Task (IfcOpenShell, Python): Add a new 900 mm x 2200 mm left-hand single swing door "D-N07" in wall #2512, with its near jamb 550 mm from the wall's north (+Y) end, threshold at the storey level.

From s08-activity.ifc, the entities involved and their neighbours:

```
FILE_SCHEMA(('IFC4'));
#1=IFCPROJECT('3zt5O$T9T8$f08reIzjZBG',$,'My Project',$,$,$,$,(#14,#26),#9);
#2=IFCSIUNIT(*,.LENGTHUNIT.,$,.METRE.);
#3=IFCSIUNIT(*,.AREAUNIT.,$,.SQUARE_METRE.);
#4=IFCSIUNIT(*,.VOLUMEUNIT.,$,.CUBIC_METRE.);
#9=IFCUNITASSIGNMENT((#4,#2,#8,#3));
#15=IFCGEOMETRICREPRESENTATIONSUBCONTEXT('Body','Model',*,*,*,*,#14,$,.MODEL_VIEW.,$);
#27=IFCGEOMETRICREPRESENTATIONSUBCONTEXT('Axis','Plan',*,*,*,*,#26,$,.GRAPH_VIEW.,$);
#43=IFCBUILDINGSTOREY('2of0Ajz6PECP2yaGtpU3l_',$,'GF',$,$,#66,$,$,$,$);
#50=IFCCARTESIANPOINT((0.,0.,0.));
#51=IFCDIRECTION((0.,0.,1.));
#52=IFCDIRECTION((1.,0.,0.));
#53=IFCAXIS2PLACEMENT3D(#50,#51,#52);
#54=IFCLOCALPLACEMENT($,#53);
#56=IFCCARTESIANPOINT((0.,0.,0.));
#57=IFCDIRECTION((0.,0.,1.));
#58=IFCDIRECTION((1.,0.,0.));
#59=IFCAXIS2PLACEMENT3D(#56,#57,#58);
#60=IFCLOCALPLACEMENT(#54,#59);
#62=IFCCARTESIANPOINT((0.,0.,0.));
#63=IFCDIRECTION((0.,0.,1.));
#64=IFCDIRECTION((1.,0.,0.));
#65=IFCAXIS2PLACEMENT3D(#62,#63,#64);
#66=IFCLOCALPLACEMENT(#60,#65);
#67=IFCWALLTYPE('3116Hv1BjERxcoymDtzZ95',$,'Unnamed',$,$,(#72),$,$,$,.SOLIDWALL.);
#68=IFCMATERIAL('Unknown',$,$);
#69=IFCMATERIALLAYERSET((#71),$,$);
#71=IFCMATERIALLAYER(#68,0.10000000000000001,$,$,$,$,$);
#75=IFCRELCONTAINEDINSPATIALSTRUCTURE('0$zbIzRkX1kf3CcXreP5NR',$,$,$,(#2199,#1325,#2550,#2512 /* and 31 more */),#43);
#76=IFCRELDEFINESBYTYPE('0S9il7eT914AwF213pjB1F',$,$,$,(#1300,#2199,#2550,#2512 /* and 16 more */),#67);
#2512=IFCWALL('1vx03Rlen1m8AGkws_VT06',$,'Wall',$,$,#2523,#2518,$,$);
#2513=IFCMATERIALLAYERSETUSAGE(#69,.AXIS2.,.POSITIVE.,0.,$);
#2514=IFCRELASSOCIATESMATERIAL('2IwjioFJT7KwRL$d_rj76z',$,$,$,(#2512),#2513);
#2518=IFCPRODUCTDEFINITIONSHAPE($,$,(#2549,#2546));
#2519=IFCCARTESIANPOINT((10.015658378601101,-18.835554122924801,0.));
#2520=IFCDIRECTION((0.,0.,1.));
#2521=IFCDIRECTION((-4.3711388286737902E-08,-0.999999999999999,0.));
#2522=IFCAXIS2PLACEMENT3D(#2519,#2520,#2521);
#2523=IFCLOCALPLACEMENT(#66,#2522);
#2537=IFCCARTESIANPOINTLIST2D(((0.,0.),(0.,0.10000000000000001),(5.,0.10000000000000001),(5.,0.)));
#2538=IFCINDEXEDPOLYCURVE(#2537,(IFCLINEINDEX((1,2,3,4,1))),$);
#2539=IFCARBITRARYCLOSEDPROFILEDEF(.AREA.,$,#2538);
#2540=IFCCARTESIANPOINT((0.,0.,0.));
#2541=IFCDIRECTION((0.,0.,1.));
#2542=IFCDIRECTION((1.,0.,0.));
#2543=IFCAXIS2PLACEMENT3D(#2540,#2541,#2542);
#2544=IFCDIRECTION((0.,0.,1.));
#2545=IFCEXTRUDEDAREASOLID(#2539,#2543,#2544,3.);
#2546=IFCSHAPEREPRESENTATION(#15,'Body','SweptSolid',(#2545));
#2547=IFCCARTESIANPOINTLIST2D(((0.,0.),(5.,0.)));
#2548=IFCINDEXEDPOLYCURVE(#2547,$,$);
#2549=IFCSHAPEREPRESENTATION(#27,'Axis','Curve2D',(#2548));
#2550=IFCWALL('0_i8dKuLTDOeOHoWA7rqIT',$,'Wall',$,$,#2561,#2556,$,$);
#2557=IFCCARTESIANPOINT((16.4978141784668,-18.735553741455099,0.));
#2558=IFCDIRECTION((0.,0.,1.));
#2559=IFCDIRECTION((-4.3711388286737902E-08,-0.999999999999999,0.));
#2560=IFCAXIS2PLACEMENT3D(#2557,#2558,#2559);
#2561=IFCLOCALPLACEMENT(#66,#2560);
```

```python
import numpy as np
import ifcopenshell
import ifcopenshell.api.feature
import ifcopenshell.api.geometry
import ifcopenshell.api.root
import ifcopenshell.api.spatial
import ifcopenshell.geom
import ifcopenshell.util.element
import ifcopenshell.util.placement
import ifcopenshell.util.representation
import ifcopenshell.util.shape
import ifcopenshell.util.unit

model = ifcopenshell.open("s08-activity.ifc")
unit_scale = ifcopenshell.util.unit.calculate_unit_scale(model)
settings = ifcopenshell.geom.settings()


def volume(element):
    """Net volume in cubic metres, openings subtracted."""
    shape = ifcopenshell.geom.create_shape(settings, element)
    return ifcopenshell.util.shape.get_volume(shape.geometry)


wall = model.by_id(2512)
storey = ifcopenshell.util.element.get_container(wall, ifc_class="IfcBuildingStorey")
context = ifcopenshell.util.representation.get_context(model, "Model", "Body", "MODEL_VIEW")
before = volume(wall)

width, height, from_end, sill = 0.9, 2.2, 0.55, 0.0  # metres

# The wall runs along its own X axis, and the end named is its -X end.
wall_shape = ifcopenshell.geom.create_shape(settings, wall)
x, y, z = ifcopenshell.util.shape.get_vertices(wall_shape.geometry).T
start = x.min() + from_end
face, thickness = float(y.min()), float(y.max() - y.min())
wall_matrix = ifcopenshell.util.placement.get_local_placement(wall.ObjectPlacement)
level = ifcopenshell.util.placement.get_local_placement(storey.ObjectPlacement)[2, 3]


def in_wall(x, y):
    """Placement at x, y metres in the wall's axes, at sill height."""
    matrix = wall_matrix.copy()
    matrix[:, 3] = wall_matrix @ np.array([x / unit_scale, y / unit_scale, 0.0, 1.0])
    matrix[2, 3] = level + sill / unit_scale
    return matrix


# Opening: a box that overshoots both wall faces by 50 mm.
opening = ifcopenshell.api.root.create_entity(model, ifc_class="IfcOpeningElement", predefined_type="OPENING")
box = ifcopenshell.api.geometry.add_wall_representation(
    model, context=context, length=width, height=height, thickness=thickness + 0.1
)
ifcopenshell.api.geometry.assign_representation(model, product=opening, representation=box)
ifcopenshell.api.geometry.edit_object_placement(model, product=opening, matrix=in_wall(start, face - 0.05), is_si=False)
ifcopenshell.api.feature.add_feature(model, feature=opening, element=wall)

door = ifcopenshell.api.root.create_entity(model, ifc_class="IfcDoor", name="D-N07", predefined_type="DOOR")
door.OverallWidth, door.OverallHeight = width / unit_scale, height / unit_scale
door.OperationType = "SINGLE_SWING_LEFT"
body = ifcopenshell.api.geometry.add_door_representation(
    model,
    context=context,
    overall_width=door.OverallWidth,
    overall_height=door.OverallHeight,
    operation_type="SINGLE_SWING_LEFT",
    lining_properties={"LiningDepth": thickness / unit_scale, "ThresholdDepth": thickness / unit_scale},
)
ifcopenshell.api.geometry.assign_representation(model, product=door, representation=body)
ifcopenshell.api.spatial.assign_container(model, products=[door], relating_structure=storey)
ifcopenshell.api.feature.add_filling(model, opening=opening, element=door)

# The lining spans the wall, so the door starts at the wall face.
ifcopenshell.api.geometry.edit_object_placement(model, product=door, matrix=in_wall(start, face), is_si=False)

after = volume(wall)

print(f"wall volume {before:.3f} -> {after:.3f} m3")

model.write("s08-activity-out.ifc")
```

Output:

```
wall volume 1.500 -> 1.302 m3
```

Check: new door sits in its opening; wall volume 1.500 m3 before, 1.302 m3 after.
